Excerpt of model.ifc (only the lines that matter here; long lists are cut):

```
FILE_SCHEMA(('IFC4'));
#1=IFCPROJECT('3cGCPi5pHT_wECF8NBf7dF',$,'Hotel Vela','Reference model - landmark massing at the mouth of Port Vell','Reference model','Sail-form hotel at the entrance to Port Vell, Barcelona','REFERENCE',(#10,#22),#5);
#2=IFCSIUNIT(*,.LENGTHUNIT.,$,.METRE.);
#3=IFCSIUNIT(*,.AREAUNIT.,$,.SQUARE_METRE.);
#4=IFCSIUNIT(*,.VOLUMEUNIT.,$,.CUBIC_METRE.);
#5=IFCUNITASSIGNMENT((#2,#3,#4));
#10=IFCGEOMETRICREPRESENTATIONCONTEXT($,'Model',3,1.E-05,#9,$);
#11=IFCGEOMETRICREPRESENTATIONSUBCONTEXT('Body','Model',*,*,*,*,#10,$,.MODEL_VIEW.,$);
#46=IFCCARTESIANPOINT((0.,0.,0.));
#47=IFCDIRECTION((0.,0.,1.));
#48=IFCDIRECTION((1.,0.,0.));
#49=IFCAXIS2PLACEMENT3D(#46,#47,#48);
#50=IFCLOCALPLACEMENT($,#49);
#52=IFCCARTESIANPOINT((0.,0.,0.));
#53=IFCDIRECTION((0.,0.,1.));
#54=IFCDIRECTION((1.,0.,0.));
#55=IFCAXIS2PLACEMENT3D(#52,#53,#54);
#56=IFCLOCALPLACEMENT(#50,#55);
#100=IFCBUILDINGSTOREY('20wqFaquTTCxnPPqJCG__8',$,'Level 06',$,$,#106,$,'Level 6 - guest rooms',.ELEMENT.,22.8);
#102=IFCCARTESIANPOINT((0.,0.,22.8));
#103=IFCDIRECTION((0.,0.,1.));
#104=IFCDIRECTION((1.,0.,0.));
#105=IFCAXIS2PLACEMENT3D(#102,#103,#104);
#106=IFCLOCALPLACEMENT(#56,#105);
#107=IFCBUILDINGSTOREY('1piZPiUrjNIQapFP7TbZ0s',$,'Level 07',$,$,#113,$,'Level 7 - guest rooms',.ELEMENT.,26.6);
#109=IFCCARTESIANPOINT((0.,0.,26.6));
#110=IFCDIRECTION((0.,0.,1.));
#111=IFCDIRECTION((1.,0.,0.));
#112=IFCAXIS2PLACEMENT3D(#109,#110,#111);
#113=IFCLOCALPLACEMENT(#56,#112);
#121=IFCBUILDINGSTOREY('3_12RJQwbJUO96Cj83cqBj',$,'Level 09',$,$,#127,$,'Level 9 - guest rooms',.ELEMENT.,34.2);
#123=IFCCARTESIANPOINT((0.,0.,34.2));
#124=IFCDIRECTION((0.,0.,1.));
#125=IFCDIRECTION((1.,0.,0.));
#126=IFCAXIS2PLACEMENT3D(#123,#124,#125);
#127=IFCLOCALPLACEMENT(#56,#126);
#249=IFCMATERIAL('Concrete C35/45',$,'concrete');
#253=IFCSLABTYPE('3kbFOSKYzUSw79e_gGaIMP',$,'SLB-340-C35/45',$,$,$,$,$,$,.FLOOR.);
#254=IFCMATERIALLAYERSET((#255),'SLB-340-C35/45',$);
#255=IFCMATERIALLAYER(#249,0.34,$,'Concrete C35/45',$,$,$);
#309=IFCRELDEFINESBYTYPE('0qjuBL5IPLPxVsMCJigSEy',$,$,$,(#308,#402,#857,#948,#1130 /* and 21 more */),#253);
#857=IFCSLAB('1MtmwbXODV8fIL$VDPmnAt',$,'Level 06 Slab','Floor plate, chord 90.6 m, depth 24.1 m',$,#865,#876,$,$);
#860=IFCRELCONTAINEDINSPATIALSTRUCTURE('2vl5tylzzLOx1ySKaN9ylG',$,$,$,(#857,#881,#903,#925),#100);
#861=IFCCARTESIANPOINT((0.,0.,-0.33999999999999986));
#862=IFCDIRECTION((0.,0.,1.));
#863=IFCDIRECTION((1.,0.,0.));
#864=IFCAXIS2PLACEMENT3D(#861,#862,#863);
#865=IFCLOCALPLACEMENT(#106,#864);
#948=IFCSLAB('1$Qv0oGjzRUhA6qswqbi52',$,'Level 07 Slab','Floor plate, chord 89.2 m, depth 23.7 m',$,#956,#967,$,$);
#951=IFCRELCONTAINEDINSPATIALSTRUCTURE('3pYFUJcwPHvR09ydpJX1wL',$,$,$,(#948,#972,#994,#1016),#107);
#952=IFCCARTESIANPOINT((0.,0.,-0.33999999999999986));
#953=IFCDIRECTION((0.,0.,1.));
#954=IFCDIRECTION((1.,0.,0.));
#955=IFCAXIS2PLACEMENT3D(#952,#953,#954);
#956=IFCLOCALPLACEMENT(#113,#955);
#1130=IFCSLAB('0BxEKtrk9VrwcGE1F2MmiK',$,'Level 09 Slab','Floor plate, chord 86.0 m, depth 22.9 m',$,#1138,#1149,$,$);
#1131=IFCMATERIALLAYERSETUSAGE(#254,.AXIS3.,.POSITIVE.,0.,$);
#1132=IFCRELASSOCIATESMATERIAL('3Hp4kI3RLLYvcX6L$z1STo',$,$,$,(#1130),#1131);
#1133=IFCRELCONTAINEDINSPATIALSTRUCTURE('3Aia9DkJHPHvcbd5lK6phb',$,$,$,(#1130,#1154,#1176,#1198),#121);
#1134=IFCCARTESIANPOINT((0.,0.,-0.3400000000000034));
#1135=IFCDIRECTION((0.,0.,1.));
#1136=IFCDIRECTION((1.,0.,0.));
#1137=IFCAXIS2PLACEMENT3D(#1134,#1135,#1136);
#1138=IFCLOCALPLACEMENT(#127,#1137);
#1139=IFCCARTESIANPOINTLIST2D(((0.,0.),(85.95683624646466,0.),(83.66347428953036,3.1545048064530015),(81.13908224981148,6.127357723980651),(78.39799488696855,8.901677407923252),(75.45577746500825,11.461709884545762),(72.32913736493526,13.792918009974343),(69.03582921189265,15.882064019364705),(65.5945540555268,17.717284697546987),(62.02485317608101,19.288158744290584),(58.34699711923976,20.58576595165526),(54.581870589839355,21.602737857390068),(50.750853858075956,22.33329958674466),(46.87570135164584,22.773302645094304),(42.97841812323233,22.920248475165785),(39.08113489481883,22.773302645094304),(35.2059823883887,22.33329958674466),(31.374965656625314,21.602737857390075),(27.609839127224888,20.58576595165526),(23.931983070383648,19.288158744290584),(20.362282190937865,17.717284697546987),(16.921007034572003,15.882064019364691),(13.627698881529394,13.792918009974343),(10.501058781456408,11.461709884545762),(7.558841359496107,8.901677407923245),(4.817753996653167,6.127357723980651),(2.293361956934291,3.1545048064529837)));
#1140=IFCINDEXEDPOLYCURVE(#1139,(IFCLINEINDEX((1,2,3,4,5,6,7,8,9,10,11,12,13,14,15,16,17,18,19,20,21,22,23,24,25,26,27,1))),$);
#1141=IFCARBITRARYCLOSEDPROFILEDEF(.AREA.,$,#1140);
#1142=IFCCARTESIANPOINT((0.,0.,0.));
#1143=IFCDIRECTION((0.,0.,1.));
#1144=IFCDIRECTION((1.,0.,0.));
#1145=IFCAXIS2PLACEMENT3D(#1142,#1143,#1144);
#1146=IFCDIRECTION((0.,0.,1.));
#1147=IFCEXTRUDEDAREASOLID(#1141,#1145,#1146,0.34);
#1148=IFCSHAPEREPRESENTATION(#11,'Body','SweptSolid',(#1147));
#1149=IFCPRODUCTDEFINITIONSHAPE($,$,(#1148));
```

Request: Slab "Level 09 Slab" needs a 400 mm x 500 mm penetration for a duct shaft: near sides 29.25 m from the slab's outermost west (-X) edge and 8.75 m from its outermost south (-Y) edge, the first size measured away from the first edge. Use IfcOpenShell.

```python
import numpy as np
import ifcopenshell
import ifcopenshell.api.feature
import ifcopenshell.api.geometry
import ifcopenshell.api.root
import ifcopenshell.geom
import ifcopenshell.util.placement
import ifcopenshell.util.representation
import ifcopenshell.util.shape
import ifcopenshell.util.unit

model = ifcopenshell.open("model.ifc")
unit_scale = ifcopenshell.util.unit.calculate_unit_scale(model)
settings = ifcopenshell.geom.settings()


def volume(element):
    """Net volume in cubic metres, openings subtracted."""
    shape = ifcopenshell.geom.create_shape(settings, element)
    return ifcopenshell.util.shape.get_volume(shape.geometry)


slab = model.by_guid("0BxEKtrk9VrwcGE1F2MmiK")
before = volume(slab)

# Extent in the slab's own axes, in metres. The edges named are its -X and -Y sides.
slab_shape = ifcopenshell.geom.create_shape(settings, slab)
vertices = ifcopenshell.util.shape.get_vertices(slab_shape.geometry)
x_min, y_min, bottom = vertices.min(axis=0)
top = vertices[:, 2].max()

opening = ifcopenshell.api.root.create_entity(model, ifc_class="IfcOpeningElement", name="Duct shaft opening", predefined_type="OPENING")
context = ifcopenshell.util.representation.get_context(model, "Model", "Body", "MODEL_VIEW")
width, depth = 0.4, 0.5
outline = [(0.0, 0.0), (width, 0.0), (width, depth), (0.0, depth), (0.0, 0.0)]
# Overshoot both faces by 50 mm so the cut is clean.
shape = ifcopenshell.api.geometry.add_slab_representation(
    model, context=context, depth=top - bottom + 0.1, polyline=outline
)
ifcopenshell.api.geometry.assign_representation(model, product=opening, representation=shape)

matrix = ifcopenshell.util.placement.get_local_placement(slab.ObjectPlacement)
matrix[:, 3] = matrix @ np.append(np.array([x_min + 29.25, y_min + 8.75, bottom - 0.05]) / unit_scale, 1.0)
ifcopenshell.api.geometry.edit_object_placement(model, product=opening, matrix=matrix, is_si=False)
ifcopenshell.api.feature.add_feature(model, feature=opening, element=slab)

after = volume(slab)

print(f"slab volume {before:.3f} -> {after:.3f} m3")

model.write("model-out.ifc")
```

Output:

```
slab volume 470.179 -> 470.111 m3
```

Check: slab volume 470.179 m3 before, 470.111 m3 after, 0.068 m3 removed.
